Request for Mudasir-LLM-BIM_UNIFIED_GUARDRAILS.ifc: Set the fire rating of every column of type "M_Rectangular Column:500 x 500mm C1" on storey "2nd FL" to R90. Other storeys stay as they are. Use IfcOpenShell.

First a look at what the model holds.

```python
import ifcopenshell
import ifcopenshell.util.element

model = ifcopenshell.open("Mudasir-LLM-BIM_UNIFIED_GUARDRAILS.ifc")
print(model.schema)
storey = next(s for s in model.by_type("IfcBuildingStorey") if s.Name == "2nd FL")
columns = [e for e in ifcopenshell.util.element.get_decomposition(storey) if e.is_a("IfcColumn")]
seen = {}
for e in columns:
    element_type = ifcopenshell.util.element.get_type(e)
    key = (element_type.Name if element_type != e and element_type else None, ifcopenshell.util.element.get_pset(e, "Pset_ColumnCommon", "FireRating"))
    seen[key] = seen.get(key, 0) + 1
for (name, value), count in sorted(seen.items(), key=str):
    print(count, "x", name, "|", value)
```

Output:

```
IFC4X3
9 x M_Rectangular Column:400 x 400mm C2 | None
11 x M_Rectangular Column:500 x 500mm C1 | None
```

```python
import ifcopenshell
import ifcopenshell.api.pset
import ifcopenshell.util.element

model = ifcopenshell.open("Mudasir-LLM-BIM_UNIFIED_GUARDRAILS.ifc")

storey = next(s for s in model.by_type("IfcBuildingStorey") if s.Name == "2nd FL")
columns = [e for e in ifcopenshell.util.element.get_decomposition(storey) if e.is_a("IfcColumn")]

count = 0
for e in columns:
    element_type = ifcopenshell.util.element.get_type(e)
    if element_type in (None, e) or element_type.Name != "M_Rectangular Column:500 x 500mm C1":
        continue
    # add_pset returns the element's existing set when there is one.
    pset = ifcopenshell.api.pset.add_pset(model, product=e, name="Pset_ColumnCommon")
    ifcopenshell.api.pset.edit_pset(model, pset=pset, properties={"FireRating": "R90"})
    count += 1

print(count, "columns updated")

model.write("Mudasir-LLM-BIM_UNIFIED_GUARDRAILS_v2.ifc")
```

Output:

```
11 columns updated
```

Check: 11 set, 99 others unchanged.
